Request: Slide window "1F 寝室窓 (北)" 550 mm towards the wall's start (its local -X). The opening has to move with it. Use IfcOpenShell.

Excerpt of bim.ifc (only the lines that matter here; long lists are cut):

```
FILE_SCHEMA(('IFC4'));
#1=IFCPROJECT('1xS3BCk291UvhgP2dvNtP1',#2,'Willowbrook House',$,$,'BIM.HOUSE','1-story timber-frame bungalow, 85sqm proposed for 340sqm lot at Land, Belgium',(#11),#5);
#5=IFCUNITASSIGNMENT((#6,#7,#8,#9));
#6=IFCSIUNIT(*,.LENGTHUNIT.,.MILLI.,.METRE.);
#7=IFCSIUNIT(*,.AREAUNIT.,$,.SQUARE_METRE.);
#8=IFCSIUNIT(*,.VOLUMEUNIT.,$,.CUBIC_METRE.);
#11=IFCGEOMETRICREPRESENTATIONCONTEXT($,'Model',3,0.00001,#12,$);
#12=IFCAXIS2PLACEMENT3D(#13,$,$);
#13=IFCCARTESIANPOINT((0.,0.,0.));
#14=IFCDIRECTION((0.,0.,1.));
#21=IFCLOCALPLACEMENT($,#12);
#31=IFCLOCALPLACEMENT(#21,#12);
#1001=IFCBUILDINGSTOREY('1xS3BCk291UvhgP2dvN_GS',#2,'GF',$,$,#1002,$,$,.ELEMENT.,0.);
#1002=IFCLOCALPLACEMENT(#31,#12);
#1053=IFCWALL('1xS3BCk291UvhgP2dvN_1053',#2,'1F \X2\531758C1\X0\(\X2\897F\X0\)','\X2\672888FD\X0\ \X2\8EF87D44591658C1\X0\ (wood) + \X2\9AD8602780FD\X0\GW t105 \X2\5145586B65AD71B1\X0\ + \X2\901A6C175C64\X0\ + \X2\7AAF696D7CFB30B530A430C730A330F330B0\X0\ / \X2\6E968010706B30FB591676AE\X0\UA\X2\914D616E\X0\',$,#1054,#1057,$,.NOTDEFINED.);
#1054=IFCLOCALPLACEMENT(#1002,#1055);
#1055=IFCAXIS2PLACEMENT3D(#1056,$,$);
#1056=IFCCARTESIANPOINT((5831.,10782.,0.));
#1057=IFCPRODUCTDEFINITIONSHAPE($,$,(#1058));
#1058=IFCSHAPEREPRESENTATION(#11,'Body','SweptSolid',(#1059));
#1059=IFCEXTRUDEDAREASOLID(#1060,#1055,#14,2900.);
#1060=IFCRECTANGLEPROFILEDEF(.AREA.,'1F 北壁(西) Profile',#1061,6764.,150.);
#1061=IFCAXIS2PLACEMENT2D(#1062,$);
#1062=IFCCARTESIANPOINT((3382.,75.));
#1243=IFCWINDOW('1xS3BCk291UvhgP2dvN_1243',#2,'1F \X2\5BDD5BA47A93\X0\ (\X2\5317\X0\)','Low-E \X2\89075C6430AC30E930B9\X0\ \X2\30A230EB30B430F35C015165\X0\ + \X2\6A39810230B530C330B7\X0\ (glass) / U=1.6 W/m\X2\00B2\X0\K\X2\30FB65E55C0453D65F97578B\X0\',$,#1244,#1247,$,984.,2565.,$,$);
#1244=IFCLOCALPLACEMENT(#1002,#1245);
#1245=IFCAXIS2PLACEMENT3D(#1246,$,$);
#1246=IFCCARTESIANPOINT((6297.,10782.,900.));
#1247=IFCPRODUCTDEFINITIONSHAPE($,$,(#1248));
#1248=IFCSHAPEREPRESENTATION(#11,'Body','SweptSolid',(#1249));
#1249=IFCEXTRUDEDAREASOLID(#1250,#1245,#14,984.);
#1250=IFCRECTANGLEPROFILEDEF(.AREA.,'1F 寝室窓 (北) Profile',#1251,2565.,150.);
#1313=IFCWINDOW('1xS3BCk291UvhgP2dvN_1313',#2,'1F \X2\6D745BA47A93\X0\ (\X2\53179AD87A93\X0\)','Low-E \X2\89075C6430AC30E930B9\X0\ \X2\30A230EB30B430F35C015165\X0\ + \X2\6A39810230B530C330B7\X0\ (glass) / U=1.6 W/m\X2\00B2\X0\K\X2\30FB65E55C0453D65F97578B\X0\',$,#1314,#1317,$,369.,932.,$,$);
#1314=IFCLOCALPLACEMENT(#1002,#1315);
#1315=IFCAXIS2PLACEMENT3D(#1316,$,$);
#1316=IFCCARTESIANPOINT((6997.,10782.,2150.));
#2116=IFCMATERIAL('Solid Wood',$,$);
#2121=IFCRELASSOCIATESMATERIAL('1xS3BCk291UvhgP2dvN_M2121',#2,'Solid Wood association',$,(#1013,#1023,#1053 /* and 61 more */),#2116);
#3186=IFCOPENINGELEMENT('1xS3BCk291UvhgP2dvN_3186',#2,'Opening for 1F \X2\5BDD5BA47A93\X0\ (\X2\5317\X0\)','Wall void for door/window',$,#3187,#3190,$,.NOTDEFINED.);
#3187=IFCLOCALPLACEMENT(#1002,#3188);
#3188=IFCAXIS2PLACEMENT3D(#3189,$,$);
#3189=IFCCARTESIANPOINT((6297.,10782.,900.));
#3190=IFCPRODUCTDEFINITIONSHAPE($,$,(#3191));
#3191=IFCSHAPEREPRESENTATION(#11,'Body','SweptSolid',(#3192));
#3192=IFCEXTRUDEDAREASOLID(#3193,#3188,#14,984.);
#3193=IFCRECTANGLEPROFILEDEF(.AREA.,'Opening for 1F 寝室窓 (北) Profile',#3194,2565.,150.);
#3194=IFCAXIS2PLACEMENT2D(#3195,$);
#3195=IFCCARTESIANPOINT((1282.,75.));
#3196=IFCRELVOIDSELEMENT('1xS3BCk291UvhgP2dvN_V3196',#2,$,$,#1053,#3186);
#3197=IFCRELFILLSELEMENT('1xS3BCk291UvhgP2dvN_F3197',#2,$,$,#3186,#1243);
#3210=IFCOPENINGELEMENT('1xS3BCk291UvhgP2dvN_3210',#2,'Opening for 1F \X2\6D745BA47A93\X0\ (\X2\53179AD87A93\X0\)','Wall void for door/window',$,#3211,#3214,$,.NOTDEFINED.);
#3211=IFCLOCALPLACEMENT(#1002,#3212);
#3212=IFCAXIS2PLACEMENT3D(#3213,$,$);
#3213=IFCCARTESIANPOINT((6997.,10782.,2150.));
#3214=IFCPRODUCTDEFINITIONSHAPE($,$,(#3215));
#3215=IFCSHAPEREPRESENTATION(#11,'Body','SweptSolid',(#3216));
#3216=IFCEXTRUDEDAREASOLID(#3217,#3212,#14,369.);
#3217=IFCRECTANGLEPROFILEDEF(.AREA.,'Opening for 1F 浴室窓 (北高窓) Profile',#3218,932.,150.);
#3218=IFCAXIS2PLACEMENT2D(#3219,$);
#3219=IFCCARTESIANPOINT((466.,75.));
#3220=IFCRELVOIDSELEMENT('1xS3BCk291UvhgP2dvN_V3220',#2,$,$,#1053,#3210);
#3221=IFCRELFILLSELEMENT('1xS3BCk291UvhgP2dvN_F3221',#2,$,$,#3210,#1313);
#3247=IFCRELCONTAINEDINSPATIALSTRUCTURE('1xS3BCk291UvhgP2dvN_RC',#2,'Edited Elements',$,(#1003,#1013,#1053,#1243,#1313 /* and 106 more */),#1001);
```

```python
import ifcopenshell
import ifcopenshell.api.geometry
import ifcopenshell.util.placement

model = ifcopenshell.open("bim.ifc")

window = model.by_guid("1xS3BCk291UvhgP2dvN_1243")
opening = window.FillsVoids[0].RelatingOpeningElement
wall = opening.VoidsElements[0].RelatingBuildingElement

wall_matrix = ifcopenshell.util.placement.get_local_placement(wall.ObjectPlacement)
shift = wall_matrix[:3, 0] * -550.0
before = ifcopenshell.util.placement.get_local_placement(window.ObjectPlacement)[:3, 3].copy()

# The window is not placed relative to its opening, so move both.
for product in (opening, window):
    matrix = ifcopenshell.util.placement.get_local_placement(product.ObjectPlacement)
    matrix[:3, 3] += shift
    ifcopenshell.api.geometry.edit_object_placement(model, product=product, matrix=matrix, is_si=False)

after = ifcopenshell.util.placement.get_local_placement(window.ObjectPlacement)[:3, 3]
print("window moved by", (after - before).round(3) + 0.0)

model.write("bim_v2.ifc")
```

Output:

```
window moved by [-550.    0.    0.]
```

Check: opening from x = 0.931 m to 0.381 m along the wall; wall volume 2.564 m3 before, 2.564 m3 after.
